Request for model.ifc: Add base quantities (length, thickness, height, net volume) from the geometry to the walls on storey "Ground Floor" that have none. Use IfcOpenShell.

First a look at what the model holds.

```python
import ifcopenshell
import ifcopenshell.util.element
import ifcopenshell.util.unit

model = ifcopenshell.open("model.ifc")
print(model.schema)
for unit_type in ("LENGTHUNIT", "AREAUNIT", "VOLUMEUNIT"):
    print(unit_type, ifcopenshell.util.unit.calculate_unit_scale(model, unit_type))
storey = next(s for s in model.by_type("IfcBuildingStorey") if s.Name == "Ground Floor")
walls = [e for e in ifcopenshell.util.element.get_decomposition(storey) if e.is_a("IfcWall")]
for e in sorted(walls, key=lambda e: e.id()):
    print(e.id(), e.is_a(), e.Name, list(ifcopenshell.util.element.get_psets(e, qtos_only=True)), sep=" | ")
```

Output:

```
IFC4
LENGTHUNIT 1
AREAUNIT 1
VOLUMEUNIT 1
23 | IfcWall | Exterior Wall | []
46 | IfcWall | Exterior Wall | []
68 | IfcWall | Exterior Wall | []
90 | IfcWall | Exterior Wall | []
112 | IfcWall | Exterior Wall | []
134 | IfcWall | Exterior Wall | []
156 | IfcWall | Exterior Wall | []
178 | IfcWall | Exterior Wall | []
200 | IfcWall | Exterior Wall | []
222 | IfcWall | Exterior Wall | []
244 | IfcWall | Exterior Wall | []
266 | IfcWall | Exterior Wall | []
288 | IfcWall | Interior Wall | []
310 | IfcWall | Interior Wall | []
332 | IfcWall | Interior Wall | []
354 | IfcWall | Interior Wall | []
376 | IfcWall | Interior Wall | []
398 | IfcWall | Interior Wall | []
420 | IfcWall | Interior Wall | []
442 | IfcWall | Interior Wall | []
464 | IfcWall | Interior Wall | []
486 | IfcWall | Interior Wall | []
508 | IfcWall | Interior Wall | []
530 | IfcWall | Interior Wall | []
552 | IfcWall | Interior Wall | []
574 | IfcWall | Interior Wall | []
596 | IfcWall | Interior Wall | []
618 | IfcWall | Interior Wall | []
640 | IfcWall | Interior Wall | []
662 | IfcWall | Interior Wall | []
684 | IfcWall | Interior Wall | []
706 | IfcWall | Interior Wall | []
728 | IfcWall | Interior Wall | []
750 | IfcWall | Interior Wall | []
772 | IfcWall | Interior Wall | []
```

```python
import ifcopenshell
import ifcopenshell.api.pset
import ifcopenshell.geom
import ifcopenshell.util.element
import ifcopenshell.util.shape
import ifcopenshell.util.unit

model = ifcopenshell.open("model.ifc")
unit_scale = ifcopenshell.util.unit.calculate_unit_scale(model)
volume_scale = ifcopenshell.util.unit.calculate_unit_scale(model, "VOLUMEUNIT")
settings = ifcopenshell.geom.settings()

storey = next(s for s in model.by_type("IfcBuildingStorey") if s.Name == "Ground Floor")
walls = [e for e in ifcopenshell.util.element.get_decomposition(storey) if e.is_a("IfcWall")]

for e in sorted(walls, key=lambda e: e.id()):
    if ifcopenshell.util.element.get_psets(e, qtos_only=True, should_inherit=False):
        continue
    # Geometry comes back in metres, in the element's own axes.
    shape = ifcopenshell.geom.create_shape(settings, e)
    values = {
        "Length": ifcopenshell.util.shape.get_x(shape.geometry) / unit_scale,
        "Width": ifcopenshell.util.shape.get_y(shape.geometry) / unit_scale,
        "Height": ifcopenshell.util.shape.get_z(shape.geometry) / unit_scale,
        "NetVolume": ifcopenshell.util.shape.get_volume(shape.geometry) / volume_scale,
    }
    qto = ifcopenshell.api.pset.add_qto(model, product=e, name="Qto_WallBaseQuantities")
    ifcopenshell.api.pset.edit_qto(model, qto=qto, properties=values)
    print(e.id(), {k: round(v, 3) for k, v in values.items()})

model.write("model_edited.ifc")
```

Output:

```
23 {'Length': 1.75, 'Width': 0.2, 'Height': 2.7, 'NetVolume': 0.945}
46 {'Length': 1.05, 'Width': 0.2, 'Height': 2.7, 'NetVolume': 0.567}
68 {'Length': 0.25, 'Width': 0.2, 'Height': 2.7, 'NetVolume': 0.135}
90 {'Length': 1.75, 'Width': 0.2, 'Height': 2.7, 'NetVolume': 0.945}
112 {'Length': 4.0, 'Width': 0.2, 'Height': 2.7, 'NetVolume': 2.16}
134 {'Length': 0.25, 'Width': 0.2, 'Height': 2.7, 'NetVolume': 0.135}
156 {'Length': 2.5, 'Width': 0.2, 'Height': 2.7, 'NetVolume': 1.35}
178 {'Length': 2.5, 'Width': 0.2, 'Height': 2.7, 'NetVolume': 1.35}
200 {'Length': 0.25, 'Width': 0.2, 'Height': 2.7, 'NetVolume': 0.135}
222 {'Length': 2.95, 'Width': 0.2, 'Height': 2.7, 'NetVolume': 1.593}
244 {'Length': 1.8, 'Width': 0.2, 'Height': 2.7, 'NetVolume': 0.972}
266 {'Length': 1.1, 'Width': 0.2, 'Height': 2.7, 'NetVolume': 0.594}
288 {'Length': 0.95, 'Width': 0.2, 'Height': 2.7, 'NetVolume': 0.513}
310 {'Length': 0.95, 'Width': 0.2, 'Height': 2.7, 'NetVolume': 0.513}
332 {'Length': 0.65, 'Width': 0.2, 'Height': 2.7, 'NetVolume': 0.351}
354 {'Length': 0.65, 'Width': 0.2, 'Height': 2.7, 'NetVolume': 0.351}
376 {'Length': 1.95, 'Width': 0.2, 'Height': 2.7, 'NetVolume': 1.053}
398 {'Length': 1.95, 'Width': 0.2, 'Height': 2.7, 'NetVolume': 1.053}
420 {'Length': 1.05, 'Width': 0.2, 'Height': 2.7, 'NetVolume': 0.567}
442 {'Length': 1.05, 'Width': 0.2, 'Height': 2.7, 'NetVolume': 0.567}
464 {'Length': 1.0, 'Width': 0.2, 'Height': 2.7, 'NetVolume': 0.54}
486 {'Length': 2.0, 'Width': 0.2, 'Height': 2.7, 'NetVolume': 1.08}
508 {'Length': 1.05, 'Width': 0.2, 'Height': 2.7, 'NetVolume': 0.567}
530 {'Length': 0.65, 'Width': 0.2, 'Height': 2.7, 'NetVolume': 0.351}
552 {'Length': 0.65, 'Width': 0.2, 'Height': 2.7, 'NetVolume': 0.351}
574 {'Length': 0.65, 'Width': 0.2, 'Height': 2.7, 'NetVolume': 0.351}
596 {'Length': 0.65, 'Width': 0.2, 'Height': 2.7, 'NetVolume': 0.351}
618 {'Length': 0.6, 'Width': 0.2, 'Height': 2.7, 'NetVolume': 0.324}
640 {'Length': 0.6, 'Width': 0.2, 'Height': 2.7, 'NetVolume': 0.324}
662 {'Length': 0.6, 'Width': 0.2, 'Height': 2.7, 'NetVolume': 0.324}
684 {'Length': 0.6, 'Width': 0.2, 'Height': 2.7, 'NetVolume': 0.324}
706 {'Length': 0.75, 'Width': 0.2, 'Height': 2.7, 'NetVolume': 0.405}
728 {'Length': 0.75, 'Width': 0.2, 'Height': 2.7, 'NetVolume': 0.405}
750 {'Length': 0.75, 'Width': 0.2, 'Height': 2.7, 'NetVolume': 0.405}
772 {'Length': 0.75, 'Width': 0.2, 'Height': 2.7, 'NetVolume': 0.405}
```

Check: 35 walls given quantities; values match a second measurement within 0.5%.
